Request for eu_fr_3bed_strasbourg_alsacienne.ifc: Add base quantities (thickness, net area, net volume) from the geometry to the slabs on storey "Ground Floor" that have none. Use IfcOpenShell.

First a look at what the model holds.

```python
import ifcopenshell
import ifcopenshell.util.element
import ifcopenshell.util.unit

model = ifcopenshell.open("eu_fr_3bed_strasbourg_alsacienne.ifc")
print(model.schema)
for unit_type in ("LENGTHUNIT", "AREAUNIT", "VOLUMEUNIT"):
    print(unit_type, ifcopenshell.util.unit.calculate_unit_scale(model, unit_type))
storey = next(s for s in model.by_type("IfcBuildingStorey") if s.Name == "Ground Floor")
slabs = [e for e in ifcopenshell.util.element.get_decomposition(storey) if e.is_a("IfcSlab")]
for e in sorted(slabs, key=lambda e: e.id()):
    print(e.id(), e.is_a(), e.Name, list(ifcopenshell.util.element.get_psets(e, qtos_only=True)), sep=" | ")
```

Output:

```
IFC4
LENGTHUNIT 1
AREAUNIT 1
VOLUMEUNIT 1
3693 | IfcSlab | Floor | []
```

```python
import ifcopenshell
import ifcopenshell.api.pset
import ifcopenshell.geom
import ifcopenshell.util.element
import ifcopenshell.util.shape
import ifcopenshell.util.unit

model = ifcopenshell.open("eu_fr_3bed_strasbourg_alsacienne.ifc")
unit_scale = ifcopenshell.util.unit.calculate_unit_scale(model)
area_scale = ifcopenshell.util.unit.calculate_unit_scale(model, "AREAUNIT")
volume_scale = ifcopenshell.util.unit.calculate_unit_scale(model, "VOLUMEUNIT")
settings = ifcopenshell.geom.settings()

storey = next(s for s in model.by_type("IfcBuildingStorey") if s.Name == "Ground Floor")
slabs = [e for e in ifcopenshell.util.element.get_decomposition(storey) if e.is_a("IfcSlab")]

for e in sorted(slabs, key=lambda e: e.id()):
    if ifcopenshell.util.element.get_psets(e, qtos_only=True, should_inherit=False):
        continue
    # Geometry comes back in metres, in the element's own axes.
    shape = ifcopenshell.geom.create_shape(settings, e)
    values = {
        "Width": ifcopenshell.util.shape.get_z(shape.geometry) / unit_scale,
        "NetArea": ifcopenshell.util.shape.get_footprint_area(shape.geometry) / area_scale,
        "NetVolume": ifcopenshell.util.shape.get_volume(shape.geometry) / volume_scale,
    }
    qto = ifcopenshell.api.pset.add_qto(model, product=e, name="Qto_SlabBaseQuantities")
    ifcopenshell.api.pset.edit_qto(model, qto=qto, properties=values)
    print(e.id(), {k: round(v, 3) for k, v in values.items()})

model.write("eu_fr_3bed_strasbourg_alsacienne_v2.ifc")
```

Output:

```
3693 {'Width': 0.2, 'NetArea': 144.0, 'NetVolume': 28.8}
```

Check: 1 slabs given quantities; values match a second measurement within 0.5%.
